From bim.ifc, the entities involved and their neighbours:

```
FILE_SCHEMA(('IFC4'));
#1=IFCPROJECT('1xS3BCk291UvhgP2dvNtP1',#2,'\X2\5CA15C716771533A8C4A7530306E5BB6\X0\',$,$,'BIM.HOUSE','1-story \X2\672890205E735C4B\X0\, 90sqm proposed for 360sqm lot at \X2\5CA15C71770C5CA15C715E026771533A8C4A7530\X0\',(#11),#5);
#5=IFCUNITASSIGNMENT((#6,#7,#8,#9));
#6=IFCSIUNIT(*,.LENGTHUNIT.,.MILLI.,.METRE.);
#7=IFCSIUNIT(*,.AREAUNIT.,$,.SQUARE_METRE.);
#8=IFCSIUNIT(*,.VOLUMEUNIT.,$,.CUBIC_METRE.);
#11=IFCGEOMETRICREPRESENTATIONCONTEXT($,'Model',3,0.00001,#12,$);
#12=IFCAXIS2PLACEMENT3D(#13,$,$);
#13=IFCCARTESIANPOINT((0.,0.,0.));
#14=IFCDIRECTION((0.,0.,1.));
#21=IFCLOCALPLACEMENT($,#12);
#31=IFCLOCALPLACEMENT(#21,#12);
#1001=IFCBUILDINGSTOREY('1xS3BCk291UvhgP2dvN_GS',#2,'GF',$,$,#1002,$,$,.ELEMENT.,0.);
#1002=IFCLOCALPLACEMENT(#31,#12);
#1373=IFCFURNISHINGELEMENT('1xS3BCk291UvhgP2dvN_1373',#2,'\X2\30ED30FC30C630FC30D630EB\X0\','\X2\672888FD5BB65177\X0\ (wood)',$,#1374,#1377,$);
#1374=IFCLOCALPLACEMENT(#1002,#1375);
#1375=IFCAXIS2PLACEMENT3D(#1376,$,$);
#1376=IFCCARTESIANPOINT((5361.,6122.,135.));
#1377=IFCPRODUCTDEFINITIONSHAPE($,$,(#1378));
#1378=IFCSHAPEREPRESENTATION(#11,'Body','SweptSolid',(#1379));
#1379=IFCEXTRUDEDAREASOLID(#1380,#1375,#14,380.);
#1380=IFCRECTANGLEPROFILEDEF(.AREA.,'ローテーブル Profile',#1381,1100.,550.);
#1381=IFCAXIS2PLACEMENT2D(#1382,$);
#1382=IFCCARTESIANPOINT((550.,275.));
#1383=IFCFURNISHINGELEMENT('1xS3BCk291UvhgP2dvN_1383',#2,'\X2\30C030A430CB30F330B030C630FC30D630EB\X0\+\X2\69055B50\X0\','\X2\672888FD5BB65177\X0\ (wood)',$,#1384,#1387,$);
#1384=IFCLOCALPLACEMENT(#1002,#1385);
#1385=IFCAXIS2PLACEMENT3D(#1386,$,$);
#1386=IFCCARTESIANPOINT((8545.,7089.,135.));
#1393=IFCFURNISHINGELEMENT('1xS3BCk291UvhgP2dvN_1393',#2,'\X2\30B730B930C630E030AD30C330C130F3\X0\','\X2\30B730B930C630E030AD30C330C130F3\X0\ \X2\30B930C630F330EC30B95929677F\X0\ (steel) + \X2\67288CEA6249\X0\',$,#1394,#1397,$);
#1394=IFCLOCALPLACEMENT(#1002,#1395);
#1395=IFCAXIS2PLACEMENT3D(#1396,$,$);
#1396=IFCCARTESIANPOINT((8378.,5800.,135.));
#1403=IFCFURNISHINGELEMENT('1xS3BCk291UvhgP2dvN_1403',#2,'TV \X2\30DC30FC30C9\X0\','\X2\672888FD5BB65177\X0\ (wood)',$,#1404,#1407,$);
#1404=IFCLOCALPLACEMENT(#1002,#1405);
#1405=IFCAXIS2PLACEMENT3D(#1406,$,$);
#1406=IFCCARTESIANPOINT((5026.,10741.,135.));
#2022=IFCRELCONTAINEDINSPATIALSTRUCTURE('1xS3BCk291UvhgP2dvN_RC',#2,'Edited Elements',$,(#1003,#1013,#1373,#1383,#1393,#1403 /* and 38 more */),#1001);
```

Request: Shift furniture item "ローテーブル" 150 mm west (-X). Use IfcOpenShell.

```python
import ifcopenshell
import ifcopenshell.api.geometry
import ifcopenshell.util.placement
import ifcopenshell.util.unit

model = ifcopenshell.open("bim.ifc")
unit_scale = ifcopenshell.util.unit.calculate_unit_scale(model)

item = model.by_guid("1xS3BCk291UvhgP2dvN_1373")
matrix = ifcopenshell.util.placement.get_local_placement(item.ObjectPlacement)
matrix[0, 3] -= 0.15 / unit_scale
ifcopenshell.api.geometry.edit_object_placement(model, product=item, matrix=matrix, is_si=False)

print(ifcopenshell.util.placement.get_local_placement(item.ObjectPlacement).round(3) + 0.0)

model.write("bim_edited.ifc")
```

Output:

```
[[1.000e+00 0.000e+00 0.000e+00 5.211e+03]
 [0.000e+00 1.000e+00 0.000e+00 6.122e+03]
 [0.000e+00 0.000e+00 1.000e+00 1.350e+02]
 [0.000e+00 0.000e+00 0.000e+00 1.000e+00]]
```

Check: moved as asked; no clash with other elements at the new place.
